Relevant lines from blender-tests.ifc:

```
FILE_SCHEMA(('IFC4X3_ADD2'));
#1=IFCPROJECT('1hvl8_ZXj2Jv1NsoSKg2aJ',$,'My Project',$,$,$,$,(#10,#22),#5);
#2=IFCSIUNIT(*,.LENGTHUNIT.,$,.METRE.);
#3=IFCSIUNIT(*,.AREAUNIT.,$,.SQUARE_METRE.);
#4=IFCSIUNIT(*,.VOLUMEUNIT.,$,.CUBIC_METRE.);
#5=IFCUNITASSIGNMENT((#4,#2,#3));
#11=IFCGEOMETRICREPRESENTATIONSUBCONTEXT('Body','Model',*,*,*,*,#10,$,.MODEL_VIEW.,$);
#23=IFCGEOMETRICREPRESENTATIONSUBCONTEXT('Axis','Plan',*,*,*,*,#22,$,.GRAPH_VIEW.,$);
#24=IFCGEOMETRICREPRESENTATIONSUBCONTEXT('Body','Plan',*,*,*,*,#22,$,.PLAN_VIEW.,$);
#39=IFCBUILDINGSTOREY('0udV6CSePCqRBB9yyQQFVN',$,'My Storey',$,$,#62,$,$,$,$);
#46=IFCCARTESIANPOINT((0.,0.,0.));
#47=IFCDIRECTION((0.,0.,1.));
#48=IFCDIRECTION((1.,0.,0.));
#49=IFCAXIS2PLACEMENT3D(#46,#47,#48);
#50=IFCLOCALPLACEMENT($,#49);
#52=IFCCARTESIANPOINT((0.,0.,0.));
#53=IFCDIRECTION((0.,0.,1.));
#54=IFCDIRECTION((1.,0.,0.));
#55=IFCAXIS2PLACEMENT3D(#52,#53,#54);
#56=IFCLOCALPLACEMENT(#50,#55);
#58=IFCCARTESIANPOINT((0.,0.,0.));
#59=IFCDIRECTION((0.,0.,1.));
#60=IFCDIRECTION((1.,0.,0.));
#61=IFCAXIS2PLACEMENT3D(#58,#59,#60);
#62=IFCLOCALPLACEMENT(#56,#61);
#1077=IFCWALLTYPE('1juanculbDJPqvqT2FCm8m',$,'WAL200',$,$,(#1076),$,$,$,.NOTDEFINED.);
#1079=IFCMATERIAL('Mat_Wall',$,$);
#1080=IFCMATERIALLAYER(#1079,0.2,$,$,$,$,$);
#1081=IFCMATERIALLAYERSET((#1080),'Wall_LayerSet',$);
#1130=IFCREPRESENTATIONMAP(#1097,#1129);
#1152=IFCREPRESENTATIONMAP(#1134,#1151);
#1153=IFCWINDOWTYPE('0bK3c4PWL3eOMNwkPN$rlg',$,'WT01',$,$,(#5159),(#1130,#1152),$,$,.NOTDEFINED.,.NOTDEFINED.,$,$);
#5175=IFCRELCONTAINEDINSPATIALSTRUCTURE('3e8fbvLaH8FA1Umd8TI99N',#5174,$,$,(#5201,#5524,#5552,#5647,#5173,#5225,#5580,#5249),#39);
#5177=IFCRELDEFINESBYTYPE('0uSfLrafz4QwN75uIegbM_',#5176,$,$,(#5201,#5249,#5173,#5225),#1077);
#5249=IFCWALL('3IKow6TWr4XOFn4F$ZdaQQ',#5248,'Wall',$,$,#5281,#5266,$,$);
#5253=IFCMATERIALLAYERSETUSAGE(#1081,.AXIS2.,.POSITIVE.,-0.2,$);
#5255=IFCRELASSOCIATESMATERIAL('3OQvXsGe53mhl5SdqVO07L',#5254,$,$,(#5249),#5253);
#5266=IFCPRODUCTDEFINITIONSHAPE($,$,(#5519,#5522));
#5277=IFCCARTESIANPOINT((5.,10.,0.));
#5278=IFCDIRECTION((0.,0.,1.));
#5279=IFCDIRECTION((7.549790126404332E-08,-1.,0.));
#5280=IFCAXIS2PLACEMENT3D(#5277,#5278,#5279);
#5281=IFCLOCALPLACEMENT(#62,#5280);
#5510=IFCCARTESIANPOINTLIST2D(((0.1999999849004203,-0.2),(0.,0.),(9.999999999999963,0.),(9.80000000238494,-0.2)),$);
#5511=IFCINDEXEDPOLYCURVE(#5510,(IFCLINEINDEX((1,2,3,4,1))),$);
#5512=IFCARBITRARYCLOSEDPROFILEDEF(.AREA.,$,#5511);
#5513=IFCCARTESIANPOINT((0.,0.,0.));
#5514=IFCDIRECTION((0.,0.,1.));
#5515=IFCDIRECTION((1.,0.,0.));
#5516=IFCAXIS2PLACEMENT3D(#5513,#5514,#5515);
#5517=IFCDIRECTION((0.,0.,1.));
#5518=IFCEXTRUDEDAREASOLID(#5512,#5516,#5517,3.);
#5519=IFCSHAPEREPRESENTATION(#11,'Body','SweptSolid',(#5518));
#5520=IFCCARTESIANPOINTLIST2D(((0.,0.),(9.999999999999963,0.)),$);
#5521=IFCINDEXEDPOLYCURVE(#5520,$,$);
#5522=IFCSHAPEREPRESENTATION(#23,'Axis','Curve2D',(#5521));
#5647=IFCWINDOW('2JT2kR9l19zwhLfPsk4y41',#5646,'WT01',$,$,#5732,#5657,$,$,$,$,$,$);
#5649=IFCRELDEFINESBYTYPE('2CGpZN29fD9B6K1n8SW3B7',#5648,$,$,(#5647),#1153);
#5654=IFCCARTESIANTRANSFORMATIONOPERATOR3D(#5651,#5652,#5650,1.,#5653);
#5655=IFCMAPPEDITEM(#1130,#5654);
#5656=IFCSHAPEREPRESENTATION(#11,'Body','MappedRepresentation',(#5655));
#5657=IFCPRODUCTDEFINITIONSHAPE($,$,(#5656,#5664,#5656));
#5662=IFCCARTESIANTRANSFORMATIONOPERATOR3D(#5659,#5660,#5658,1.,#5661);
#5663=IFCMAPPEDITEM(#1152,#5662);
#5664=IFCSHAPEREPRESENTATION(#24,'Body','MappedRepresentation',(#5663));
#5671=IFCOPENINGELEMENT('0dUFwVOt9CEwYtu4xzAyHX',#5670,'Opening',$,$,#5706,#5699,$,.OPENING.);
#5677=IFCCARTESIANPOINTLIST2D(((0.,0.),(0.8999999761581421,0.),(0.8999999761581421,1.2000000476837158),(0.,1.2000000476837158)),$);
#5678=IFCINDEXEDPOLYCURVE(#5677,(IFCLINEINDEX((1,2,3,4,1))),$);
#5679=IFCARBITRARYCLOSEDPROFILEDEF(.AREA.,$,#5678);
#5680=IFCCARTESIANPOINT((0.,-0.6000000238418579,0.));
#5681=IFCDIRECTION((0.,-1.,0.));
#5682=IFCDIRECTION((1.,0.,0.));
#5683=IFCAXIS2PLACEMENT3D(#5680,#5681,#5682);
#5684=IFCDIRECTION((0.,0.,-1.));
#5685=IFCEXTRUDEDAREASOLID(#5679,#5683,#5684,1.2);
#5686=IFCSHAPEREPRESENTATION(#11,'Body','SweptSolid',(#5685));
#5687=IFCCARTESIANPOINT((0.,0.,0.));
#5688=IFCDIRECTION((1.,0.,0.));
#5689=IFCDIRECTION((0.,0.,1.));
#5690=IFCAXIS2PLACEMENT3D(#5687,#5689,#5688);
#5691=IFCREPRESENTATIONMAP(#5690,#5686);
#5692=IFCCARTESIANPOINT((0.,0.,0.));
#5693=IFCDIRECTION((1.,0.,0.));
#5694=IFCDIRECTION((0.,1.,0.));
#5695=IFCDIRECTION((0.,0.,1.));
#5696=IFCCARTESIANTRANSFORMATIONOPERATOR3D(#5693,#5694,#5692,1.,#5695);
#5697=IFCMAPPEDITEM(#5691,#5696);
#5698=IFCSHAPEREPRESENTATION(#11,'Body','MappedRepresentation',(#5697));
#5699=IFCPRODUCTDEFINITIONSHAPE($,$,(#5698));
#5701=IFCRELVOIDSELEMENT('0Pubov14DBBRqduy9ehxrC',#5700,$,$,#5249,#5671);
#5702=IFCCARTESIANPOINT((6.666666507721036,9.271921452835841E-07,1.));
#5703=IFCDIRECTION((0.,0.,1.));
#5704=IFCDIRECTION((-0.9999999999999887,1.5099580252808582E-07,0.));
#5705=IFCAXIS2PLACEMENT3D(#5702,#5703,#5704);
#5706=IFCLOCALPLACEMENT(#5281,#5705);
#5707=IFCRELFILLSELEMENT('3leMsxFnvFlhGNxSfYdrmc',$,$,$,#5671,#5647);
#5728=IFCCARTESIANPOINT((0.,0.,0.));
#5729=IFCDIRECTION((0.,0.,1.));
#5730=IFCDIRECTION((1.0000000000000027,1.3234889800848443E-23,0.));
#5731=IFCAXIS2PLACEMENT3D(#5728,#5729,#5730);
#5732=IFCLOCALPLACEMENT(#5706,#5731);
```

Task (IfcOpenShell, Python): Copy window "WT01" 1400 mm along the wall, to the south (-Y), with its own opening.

```python
import ifcopenshell
import ifcopenshell.api.feature
import ifcopenshell.api.geometry
import ifcopenshell.api.root
import ifcopenshell.geom
import ifcopenshell.util.element
import ifcopenshell.util.placement
import ifcopenshell.util.shape
import ifcopenshell.util.unit

model = ifcopenshell.open("blender-tests.ifc")
unit_scale = ifcopenshell.util.unit.calculate_unit_scale(model)
settings = ifcopenshell.geom.settings()


def volume(element):
    """Net volume in cubic metres, openings subtracted."""
    shape = ifcopenshell.geom.create_shape(settings, element)
    return ifcopenshell.util.shape.get_volume(shape.geometry)


def reuse_history(source, copy):
    """copy_class also copies each property set's owner history, people and application; keep the originals."""
    for rel in copy.IsDefinedBy:
        if rel.is_a("IfcRelDefinesByProperties") and (history := rel.RelatingPropertyDefinition.OwnerHistory):
            rel.RelatingPropertyDefinition.OwnerHistory = source.OwnerHistory
            ifcopenshell.util.element.remove_deep2(model, history)


window = model.by_guid("2JT2kR9l19zwhLfPsk4y41")
opening = window.FillsVoids[0].RelatingOpeningElement
wall = opening.VoidsElements[0].RelatingBuildingElement
before = volume(wall)
shift = ifcopenshell.util.placement.get_local_placement(wall.ObjectPlacement)[:3, 0] * 1.4 / unit_scale

# copy_class copies the void relationship, type, container and properties, but no geometry.
new_opening = ifcopenshell.api.root.copy_class(model, product=opening)
new_opening.Representation = ifcopenshell.util.element.copy_deep(
    model, opening.Representation, exclude=["IfcGeometricRepresentationContext", "IfcRepresentationMap"]
)
reuse_history(opening, new_opening)
new_window = ifcopenshell.api.root.copy_class(model, product=window)
new_window.Representation = ifcopenshell.util.element.copy_deep(
    model, window.Representation, exclude=["IfcGeometricRepresentationContext", "IfcRepresentationMap"]
)
reuse_history(window, new_window)
ifcopenshell.api.feature.add_filling(model, opening=new_opening, element=new_window)

for old, new in ((opening, new_opening), (window, new_window)):
    matrix = ifcopenshell.util.placement.get_local_placement(old.ObjectPlacement)
    matrix[:3, 3] += shift
    ifcopenshell.api.geometry.edit_object_placement(model, product=new, matrix=matrix, is_si=False)

after = volume(wall)

print(f"wall volume {before:.3f} -> {after:.3f} m3")

model.write("blender-tests_edited.ifc")
```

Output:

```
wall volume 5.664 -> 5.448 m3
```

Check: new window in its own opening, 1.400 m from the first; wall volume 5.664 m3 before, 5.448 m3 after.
